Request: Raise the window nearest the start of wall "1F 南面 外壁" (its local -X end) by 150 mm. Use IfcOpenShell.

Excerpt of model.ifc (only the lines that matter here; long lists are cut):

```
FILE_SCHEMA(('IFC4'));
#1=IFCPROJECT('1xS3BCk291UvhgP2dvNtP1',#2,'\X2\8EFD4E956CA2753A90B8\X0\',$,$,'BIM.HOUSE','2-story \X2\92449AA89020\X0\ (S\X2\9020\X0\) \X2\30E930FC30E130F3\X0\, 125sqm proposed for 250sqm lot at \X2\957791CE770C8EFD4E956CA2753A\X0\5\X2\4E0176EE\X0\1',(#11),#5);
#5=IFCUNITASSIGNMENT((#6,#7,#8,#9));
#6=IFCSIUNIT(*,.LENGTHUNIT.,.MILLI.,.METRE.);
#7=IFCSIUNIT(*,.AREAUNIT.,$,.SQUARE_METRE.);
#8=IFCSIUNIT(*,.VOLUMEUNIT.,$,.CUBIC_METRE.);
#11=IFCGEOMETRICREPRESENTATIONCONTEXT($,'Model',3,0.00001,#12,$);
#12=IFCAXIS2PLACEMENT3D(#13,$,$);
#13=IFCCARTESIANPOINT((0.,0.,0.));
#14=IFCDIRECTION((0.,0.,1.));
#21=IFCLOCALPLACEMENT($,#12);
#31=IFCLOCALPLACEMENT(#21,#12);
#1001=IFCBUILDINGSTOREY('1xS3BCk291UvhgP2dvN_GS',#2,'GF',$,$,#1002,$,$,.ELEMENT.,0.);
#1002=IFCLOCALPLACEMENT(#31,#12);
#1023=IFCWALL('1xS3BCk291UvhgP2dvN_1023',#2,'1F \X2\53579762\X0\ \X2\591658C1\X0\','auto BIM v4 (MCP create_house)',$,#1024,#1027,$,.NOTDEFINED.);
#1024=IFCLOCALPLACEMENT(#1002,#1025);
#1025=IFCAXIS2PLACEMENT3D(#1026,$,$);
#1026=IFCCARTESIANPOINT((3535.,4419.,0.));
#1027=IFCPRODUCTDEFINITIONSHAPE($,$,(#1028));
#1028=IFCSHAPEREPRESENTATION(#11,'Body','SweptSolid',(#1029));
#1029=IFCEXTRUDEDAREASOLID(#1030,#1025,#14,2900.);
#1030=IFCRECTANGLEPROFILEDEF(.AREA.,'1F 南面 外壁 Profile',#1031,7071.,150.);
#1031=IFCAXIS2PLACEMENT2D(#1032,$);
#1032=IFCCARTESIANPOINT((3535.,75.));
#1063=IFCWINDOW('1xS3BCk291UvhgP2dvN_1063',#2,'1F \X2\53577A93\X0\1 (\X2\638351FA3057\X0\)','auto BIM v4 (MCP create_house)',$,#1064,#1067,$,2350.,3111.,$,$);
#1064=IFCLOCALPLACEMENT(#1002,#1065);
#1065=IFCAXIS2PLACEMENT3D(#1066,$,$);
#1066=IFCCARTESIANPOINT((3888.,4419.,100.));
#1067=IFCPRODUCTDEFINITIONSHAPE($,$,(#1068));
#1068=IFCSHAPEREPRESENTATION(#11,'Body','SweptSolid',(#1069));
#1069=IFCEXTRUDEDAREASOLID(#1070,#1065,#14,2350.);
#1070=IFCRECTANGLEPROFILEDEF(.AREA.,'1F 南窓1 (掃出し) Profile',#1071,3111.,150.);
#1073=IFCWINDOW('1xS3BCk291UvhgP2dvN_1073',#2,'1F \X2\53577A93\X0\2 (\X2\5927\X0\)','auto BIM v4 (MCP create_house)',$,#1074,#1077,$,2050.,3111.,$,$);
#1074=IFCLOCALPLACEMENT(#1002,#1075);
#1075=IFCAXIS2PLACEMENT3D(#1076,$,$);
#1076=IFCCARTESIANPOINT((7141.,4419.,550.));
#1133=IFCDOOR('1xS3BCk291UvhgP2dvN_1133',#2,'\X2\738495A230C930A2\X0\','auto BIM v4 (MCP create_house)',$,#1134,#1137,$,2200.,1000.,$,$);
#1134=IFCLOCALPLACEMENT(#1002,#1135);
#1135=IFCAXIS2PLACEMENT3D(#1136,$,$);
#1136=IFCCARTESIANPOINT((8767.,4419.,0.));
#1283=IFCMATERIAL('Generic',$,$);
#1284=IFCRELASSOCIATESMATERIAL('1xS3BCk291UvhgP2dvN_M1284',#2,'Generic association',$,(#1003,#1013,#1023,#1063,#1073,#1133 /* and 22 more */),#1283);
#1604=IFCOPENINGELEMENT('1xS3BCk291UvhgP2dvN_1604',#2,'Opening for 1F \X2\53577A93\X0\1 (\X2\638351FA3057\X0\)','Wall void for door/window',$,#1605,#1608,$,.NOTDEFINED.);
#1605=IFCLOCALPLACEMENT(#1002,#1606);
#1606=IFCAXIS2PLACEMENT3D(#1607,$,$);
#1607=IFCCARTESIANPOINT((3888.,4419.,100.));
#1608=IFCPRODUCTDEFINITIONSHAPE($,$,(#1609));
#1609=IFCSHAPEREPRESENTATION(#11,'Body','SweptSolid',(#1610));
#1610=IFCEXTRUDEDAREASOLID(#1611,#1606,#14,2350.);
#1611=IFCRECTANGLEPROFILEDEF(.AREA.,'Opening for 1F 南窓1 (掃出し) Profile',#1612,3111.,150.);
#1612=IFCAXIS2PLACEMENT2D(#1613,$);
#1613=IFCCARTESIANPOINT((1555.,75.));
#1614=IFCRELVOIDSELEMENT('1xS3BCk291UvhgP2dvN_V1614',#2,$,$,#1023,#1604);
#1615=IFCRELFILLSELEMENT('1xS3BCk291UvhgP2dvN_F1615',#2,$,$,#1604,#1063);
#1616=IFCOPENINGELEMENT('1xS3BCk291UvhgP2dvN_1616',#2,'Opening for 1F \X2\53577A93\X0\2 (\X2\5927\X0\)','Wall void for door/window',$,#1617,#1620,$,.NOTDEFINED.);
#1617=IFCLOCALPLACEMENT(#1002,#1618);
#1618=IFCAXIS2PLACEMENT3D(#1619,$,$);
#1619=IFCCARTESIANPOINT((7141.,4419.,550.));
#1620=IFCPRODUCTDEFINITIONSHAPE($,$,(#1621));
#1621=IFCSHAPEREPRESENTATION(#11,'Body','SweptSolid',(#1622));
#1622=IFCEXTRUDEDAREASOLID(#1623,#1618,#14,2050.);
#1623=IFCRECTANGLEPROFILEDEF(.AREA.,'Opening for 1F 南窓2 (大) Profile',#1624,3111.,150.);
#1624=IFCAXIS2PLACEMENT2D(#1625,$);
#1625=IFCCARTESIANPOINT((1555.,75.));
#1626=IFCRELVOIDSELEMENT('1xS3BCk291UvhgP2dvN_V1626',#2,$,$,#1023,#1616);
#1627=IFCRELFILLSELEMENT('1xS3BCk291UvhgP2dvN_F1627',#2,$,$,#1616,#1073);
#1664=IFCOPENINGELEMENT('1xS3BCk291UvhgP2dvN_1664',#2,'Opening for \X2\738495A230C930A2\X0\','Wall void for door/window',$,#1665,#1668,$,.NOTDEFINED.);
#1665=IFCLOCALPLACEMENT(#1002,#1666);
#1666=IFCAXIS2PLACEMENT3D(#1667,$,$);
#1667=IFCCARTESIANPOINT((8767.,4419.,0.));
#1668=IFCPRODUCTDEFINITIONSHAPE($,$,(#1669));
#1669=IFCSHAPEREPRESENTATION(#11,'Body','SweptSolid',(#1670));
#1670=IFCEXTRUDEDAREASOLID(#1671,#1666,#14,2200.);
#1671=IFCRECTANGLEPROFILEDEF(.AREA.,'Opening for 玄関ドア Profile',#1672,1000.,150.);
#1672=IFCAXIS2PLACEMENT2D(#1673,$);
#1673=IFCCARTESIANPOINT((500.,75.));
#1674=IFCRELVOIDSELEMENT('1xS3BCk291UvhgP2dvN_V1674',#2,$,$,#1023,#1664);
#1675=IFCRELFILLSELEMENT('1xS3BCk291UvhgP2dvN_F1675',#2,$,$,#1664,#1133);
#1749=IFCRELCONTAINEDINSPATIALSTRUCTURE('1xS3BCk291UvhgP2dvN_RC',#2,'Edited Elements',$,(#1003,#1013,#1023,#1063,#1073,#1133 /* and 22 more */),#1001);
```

```python
import numpy as np
import ifcopenshell
import ifcopenshell.api.geometry
import ifcopenshell.util.placement
import ifcopenshell.util.unit

model = ifcopenshell.open("model.ifc")
unit_scale = ifcopenshell.util.unit.calculate_unit_scale(model)

window = model.by_guid("1xS3BCk291UvhgP2dvN_1063")
opening = window.FillsVoids[0].RelatingOpeningElement
dz = 0.15 / unit_scale

shift = np.array([0.0, 0.0, dz])
# The window is not placed relative to its opening, so move both.
for product in (opening, window):
    matrix = ifcopenshell.util.placement.get_local_placement(product.ObjectPlacement)
    matrix[:3, 3] += shift
    ifcopenshell.api.geometry.edit_object_placement(model, product=product, matrix=matrix, is_si=False)

print(f"moved by {dz * unit_scale:+.3f} m")

model.write("model_edited.ifc")
```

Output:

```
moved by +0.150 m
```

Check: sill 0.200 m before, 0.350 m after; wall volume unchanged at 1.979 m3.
